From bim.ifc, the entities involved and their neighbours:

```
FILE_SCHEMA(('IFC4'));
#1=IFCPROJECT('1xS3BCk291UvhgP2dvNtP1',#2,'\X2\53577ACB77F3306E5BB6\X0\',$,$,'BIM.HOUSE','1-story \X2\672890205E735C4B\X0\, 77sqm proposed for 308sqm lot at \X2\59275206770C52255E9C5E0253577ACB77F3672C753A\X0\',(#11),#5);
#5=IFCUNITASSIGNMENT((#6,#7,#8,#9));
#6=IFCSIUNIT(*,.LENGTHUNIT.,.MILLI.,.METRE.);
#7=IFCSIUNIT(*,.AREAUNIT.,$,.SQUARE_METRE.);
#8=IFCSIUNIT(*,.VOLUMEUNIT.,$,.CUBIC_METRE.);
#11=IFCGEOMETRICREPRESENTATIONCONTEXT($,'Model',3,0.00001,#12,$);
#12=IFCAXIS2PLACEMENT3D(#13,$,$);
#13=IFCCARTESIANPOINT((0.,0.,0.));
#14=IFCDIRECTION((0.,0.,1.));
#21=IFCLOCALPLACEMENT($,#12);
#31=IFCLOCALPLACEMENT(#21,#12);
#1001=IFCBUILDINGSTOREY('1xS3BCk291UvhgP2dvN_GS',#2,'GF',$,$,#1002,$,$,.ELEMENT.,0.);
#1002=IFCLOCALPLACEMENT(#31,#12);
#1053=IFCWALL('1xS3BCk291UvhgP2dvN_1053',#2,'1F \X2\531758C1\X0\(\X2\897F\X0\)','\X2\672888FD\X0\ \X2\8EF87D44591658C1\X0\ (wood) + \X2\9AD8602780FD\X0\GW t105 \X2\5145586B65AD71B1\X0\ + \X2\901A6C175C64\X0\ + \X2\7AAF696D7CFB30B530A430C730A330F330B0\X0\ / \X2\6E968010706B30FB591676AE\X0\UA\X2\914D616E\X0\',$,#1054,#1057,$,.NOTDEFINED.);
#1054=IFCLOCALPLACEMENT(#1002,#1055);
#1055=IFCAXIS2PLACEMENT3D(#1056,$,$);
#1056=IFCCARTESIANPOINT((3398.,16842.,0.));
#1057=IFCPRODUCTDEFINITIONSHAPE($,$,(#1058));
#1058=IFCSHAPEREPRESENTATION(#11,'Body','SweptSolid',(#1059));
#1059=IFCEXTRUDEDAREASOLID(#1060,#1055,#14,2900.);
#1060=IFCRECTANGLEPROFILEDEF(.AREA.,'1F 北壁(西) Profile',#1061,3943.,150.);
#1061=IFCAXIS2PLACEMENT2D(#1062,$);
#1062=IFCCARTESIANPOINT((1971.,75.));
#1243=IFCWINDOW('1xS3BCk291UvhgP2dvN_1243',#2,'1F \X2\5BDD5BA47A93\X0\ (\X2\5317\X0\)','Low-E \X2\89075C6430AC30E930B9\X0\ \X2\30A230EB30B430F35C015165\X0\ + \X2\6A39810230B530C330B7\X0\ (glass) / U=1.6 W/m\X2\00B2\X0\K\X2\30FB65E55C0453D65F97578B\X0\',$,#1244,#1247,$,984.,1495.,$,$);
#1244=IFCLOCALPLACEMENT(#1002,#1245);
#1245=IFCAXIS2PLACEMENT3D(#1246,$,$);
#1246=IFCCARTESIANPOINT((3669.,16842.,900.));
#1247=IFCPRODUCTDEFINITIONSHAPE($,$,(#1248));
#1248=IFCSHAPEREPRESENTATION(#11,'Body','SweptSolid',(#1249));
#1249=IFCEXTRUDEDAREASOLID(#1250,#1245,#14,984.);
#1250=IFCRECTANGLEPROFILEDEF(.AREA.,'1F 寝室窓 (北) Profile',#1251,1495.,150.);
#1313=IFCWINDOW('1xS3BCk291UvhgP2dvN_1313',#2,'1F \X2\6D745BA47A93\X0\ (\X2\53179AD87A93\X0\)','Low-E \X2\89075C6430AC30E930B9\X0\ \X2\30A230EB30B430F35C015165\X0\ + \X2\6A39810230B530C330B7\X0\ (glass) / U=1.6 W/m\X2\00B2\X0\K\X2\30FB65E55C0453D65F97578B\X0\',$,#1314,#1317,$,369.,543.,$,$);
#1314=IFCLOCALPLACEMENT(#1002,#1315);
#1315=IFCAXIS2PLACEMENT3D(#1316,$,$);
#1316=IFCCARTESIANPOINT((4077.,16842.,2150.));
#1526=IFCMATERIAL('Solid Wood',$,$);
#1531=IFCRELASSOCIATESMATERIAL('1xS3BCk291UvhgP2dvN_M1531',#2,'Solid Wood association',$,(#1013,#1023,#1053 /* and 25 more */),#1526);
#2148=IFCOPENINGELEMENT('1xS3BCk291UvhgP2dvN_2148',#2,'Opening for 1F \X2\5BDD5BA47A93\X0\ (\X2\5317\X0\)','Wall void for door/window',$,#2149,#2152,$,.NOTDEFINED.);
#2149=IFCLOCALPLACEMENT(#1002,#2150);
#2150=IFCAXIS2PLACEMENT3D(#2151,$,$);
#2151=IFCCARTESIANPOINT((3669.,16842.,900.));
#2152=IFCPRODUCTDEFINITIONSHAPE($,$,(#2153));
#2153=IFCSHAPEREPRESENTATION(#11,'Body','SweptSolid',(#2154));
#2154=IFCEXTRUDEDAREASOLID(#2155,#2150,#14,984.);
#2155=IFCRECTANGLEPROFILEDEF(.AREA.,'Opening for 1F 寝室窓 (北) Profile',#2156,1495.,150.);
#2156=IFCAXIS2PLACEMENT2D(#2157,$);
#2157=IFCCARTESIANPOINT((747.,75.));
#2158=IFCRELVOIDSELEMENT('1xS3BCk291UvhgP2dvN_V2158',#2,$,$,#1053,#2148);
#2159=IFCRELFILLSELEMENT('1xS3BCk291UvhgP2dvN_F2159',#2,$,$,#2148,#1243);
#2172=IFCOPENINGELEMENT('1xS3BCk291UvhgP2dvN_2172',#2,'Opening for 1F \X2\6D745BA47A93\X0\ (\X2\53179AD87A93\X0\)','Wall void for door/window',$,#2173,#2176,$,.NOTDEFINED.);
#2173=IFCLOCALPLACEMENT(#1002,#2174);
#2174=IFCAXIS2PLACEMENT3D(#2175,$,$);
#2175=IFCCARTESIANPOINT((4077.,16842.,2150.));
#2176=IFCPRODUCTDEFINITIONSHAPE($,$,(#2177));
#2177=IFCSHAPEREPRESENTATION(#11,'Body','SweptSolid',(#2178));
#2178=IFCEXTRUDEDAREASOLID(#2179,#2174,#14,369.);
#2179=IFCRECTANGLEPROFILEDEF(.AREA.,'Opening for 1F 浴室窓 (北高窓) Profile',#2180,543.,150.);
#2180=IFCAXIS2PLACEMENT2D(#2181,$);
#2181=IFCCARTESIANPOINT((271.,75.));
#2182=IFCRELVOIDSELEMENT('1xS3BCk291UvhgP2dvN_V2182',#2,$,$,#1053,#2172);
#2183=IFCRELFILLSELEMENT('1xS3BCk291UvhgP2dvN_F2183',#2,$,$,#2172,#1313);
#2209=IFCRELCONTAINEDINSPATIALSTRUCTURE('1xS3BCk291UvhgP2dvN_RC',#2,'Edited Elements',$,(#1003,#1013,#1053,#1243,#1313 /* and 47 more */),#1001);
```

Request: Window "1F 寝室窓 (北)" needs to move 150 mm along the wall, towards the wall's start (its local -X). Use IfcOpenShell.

```python
import ifcopenshell
import ifcopenshell.api.geometry
import ifcopenshell.util.placement

model = ifcopenshell.open("bim.ifc")

window = model.by_guid("1xS3BCk291UvhgP2dvN_1243")
opening = window.FillsVoids[0].RelatingOpeningElement
wall = opening.VoidsElements[0].RelatingBuildingElement

wall_matrix = ifcopenshell.util.placement.get_local_placement(wall.ObjectPlacement)
shift = wall_matrix[:3, 0] * -150.0
before = ifcopenshell.util.placement.get_local_placement(window.ObjectPlacement)[:3, 3].copy()

# The window is not placed relative to its opening, so move both.
for product in (opening, window):
    matrix = ifcopenshell.util.placement.get_local_placement(product.ObjectPlacement)
    matrix[:3, 3] += shift
    ifcopenshell.api.geometry.edit_object_placement(model, product=product, matrix=matrix, is_si=False)

after = ifcopenshell.util.placement.get_local_placement(window.ObjectPlacement)[:3, 3]
print("window moved by", (after - before).round(3) + 0.0)

model.write("bim-out.ifc")
```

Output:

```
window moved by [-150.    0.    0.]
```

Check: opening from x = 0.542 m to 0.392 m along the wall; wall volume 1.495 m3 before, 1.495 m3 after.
